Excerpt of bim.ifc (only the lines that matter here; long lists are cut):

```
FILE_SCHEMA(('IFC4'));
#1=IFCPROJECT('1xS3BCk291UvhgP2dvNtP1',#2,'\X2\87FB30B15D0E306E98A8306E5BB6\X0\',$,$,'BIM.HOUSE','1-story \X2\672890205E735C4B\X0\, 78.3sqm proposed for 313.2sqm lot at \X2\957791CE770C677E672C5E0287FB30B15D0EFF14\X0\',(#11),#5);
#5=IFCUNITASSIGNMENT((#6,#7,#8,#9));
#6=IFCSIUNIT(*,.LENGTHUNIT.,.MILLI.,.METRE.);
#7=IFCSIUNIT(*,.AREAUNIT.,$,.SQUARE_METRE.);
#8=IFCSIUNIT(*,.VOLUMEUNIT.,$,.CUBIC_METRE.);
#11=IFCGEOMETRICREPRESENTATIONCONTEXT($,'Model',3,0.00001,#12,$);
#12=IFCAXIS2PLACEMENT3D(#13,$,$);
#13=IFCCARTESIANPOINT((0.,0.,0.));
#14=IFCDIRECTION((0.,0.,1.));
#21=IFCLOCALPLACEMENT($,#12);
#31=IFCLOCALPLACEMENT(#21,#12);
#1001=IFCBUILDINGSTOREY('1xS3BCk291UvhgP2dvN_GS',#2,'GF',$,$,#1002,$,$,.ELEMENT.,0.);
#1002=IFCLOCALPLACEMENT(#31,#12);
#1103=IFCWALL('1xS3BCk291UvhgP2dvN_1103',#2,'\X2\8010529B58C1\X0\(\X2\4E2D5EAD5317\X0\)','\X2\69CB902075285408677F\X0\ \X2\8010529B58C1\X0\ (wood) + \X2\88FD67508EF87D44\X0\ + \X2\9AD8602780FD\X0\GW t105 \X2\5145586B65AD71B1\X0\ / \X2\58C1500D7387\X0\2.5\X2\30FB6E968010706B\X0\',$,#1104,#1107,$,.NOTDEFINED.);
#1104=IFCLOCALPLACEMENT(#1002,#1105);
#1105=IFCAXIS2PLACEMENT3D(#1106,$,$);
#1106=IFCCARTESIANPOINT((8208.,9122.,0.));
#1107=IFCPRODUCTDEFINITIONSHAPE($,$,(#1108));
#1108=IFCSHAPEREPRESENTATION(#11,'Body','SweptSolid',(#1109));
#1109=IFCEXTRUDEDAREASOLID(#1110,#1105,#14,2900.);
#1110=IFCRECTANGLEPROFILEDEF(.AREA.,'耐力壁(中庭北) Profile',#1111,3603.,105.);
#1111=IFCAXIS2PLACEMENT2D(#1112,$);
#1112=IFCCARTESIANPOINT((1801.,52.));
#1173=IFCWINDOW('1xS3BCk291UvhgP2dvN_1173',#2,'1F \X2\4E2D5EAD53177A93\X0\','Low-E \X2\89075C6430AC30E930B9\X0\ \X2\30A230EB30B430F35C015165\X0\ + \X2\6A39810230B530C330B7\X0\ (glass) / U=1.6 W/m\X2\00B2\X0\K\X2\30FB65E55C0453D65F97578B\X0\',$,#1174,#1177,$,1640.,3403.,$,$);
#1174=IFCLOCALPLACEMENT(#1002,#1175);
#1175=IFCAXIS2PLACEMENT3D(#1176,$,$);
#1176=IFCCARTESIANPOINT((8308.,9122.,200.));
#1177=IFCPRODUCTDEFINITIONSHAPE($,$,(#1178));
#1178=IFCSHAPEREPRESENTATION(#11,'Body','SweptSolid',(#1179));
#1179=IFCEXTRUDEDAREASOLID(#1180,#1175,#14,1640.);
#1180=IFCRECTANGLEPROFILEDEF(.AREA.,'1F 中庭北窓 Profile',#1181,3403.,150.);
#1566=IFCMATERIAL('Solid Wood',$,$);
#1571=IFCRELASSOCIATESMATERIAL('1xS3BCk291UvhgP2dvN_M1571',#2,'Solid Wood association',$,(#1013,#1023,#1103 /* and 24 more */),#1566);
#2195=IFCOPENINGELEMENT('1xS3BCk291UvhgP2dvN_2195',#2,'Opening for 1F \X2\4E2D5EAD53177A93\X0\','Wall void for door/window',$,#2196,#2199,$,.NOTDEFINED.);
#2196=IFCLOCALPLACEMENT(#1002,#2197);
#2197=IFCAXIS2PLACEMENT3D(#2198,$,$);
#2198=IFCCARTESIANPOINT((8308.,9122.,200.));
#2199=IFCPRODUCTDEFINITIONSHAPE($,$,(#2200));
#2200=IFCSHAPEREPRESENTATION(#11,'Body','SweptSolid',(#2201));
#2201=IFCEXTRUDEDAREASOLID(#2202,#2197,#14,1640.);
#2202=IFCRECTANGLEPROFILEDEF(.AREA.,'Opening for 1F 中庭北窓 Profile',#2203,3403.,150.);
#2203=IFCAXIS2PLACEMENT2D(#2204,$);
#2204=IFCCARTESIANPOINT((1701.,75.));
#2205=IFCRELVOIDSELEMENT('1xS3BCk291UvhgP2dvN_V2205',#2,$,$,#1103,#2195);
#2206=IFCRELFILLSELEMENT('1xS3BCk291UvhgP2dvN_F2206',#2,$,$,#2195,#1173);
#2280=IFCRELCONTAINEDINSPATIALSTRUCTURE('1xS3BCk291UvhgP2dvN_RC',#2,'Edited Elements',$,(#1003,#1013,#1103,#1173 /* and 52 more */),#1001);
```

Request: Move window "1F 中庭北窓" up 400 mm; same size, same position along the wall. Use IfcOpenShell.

```python
import numpy as np
import ifcopenshell
import ifcopenshell.api.geometry
import ifcopenshell.util.placement
import ifcopenshell.util.unit

model = ifcopenshell.open("bim.ifc")
unit_scale = ifcopenshell.util.unit.calculate_unit_scale(model)

window = model.by_guid("1xS3BCk291UvhgP2dvN_1173")
opening = window.FillsVoids[0].RelatingOpeningElement
dz = 0.4 / unit_scale

shift = np.array([0.0, 0.0, dz])
# The window is not placed relative to its opening, so move both.
for product in (opening, window):
    matrix = ifcopenshell.util.placement.get_local_placement(product.ObjectPlacement)
    matrix[:3, 3] += shift
    ifcopenshell.api.geometry.edit_object_placement(model, product=product, matrix=matrix, is_si=False)

print(f"moved by {dz * unit_scale:+.3f} m")

model.write("bim_v2.ifc")
```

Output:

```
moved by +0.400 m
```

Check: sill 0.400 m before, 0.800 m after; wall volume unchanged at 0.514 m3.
